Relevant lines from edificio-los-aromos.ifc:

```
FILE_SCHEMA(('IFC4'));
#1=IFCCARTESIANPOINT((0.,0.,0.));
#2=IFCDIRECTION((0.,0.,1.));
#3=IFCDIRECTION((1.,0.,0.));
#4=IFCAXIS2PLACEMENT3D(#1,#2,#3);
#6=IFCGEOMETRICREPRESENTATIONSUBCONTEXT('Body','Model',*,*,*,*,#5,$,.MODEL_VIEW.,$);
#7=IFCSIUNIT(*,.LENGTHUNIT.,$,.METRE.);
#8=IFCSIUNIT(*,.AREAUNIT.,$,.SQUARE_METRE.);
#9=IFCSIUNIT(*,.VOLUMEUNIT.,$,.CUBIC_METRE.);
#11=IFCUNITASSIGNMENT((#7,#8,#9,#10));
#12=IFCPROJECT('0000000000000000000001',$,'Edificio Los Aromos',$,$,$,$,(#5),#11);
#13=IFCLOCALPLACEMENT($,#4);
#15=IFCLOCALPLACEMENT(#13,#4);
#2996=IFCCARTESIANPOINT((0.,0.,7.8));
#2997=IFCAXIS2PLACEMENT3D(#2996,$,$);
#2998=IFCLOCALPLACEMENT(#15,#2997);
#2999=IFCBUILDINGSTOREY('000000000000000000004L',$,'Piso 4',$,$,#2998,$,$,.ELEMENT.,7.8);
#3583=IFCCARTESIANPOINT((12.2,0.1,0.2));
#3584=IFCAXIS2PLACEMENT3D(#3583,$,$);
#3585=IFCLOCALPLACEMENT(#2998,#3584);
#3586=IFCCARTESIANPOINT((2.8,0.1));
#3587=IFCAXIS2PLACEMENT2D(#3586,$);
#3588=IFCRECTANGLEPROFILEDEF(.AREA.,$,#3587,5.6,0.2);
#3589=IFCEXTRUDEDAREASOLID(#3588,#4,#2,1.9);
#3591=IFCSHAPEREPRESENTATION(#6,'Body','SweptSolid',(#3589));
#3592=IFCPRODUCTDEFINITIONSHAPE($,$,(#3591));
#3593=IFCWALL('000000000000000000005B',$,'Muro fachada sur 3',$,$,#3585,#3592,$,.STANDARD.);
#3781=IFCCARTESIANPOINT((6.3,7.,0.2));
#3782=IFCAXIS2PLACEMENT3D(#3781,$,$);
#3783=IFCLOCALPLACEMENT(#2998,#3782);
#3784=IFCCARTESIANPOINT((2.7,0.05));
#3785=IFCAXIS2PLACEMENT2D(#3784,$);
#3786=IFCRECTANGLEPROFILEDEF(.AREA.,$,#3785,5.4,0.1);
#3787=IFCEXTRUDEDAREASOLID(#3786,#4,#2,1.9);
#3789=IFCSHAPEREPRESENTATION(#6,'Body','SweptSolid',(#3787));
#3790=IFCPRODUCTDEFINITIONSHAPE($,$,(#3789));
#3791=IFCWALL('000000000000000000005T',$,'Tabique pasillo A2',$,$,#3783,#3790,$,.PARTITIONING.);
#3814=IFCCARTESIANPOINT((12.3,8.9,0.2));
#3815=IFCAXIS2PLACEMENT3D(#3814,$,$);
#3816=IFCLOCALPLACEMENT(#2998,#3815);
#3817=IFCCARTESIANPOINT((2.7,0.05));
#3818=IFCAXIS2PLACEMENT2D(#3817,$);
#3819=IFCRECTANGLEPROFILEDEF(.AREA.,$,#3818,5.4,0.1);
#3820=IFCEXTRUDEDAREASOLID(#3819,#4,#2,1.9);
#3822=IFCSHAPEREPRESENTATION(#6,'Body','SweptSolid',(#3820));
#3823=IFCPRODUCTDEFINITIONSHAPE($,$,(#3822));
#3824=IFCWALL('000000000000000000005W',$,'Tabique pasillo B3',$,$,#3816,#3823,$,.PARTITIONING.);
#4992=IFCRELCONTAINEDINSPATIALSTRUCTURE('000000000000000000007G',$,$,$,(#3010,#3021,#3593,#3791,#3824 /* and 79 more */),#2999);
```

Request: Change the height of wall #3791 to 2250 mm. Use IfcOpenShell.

```python
import ifcopenshell
import ifcopenshell.geom
import ifcopenshell.util.representation
import ifcopenshell.util.shape
import ifcopenshell.util.unit

model = ifcopenshell.open("edificio-los-aromos.ifc")
unit_scale = ifcopenshell.util.unit.calculate_unit_scale(model)
settings = ifcopenshell.geom.settings()


def volume(element):
    """Net volume in cubic metres, openings subtracted."""
    shape = ifcopenshell.geom.create_shape(settings, element)
    return ifcopenshell.util.shape.get_volume(shape.geometry)


wall = model.by_guid("000000000000000000005T")
before = volume(wall)

body = ifcopenshell.util.representation.get_representation(wall, "Model", "Body")
solid = body.Items[0]
old_height = solid.Depth
solid.Depth = 2.25 / unit_scale
after = volume(wall)

print(f"height {old_height:g} -> {solid.Depth:g}, volume {before:.3f} -> {after:.3f} m3")

model.write("edificio-los-aromos_updated.ifc")
```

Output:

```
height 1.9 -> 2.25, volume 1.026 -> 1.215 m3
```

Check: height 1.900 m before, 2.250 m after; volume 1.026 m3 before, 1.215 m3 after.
